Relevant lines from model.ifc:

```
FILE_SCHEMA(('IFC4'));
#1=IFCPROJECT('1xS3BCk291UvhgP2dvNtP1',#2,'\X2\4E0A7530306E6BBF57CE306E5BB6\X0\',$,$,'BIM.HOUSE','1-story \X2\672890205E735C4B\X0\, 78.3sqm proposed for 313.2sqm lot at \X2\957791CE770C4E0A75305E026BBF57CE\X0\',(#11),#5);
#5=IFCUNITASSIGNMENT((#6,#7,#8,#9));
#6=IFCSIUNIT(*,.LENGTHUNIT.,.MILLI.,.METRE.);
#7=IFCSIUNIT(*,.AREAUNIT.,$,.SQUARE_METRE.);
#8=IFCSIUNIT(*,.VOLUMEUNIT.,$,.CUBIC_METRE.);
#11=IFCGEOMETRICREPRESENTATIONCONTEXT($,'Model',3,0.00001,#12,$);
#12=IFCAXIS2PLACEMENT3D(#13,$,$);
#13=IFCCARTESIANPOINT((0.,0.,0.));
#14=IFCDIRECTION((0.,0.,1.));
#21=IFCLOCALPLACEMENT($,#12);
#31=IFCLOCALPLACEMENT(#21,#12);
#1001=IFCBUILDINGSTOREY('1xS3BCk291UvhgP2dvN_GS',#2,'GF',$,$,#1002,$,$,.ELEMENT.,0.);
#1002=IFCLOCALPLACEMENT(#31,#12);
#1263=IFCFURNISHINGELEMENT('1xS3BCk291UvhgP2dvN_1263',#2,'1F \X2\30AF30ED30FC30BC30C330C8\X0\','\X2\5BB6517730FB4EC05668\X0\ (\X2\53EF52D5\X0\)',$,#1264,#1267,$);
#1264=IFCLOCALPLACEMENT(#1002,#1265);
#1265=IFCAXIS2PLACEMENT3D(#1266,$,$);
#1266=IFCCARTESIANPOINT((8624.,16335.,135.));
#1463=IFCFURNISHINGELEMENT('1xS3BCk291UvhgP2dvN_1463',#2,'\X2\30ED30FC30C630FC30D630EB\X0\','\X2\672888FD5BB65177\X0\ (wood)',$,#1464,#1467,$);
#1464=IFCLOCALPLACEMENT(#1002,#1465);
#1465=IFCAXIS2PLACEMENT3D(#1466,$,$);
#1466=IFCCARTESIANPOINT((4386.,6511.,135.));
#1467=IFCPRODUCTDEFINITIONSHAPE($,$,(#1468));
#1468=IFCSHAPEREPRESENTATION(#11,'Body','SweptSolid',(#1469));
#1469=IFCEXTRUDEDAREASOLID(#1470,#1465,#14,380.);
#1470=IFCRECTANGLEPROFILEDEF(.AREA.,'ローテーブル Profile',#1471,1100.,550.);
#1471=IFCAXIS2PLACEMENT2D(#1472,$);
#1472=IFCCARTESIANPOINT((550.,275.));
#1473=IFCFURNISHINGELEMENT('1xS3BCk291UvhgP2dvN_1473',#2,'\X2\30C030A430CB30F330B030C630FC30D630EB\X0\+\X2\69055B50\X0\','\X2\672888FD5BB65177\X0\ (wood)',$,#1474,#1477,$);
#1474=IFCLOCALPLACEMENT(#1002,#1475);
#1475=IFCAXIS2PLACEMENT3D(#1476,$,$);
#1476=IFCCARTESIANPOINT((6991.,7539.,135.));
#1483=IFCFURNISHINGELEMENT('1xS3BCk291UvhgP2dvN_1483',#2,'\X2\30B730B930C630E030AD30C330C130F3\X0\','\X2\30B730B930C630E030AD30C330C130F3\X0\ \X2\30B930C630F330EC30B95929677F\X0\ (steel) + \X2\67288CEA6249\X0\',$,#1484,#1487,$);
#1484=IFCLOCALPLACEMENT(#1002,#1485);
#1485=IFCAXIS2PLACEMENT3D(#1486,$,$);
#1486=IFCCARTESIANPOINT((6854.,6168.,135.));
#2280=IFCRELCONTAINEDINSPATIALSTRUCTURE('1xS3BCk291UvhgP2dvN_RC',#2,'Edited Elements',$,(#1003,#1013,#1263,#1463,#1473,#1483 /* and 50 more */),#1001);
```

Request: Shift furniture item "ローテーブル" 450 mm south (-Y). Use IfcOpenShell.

```python
import ifcopenshell
import ifcopenshell.api.geometry
import ifcopenshell.util.placement
import ifcopenshell.util.unit

model = ifcopenshell.open("model.ifc")
unit_scale = ifcopenshell.util.unit.calculate_unit_scale(model)

item = model.by_id(1463)
matrix = ifcopenshell.util.placement.get_local_placement(item.ObjectPlacement)
matrix[1, 3] -= 0.45 / unit_scale
ifcopenshell.api.geometry.edit_object_placement(model, product=item, matrix=matrix, is_si=False)

print(ifcopenshell.util.placement.get_local_placement(item.ObjectPlacement).round(3) + 0.0)

model.write("model-out.ifc")
```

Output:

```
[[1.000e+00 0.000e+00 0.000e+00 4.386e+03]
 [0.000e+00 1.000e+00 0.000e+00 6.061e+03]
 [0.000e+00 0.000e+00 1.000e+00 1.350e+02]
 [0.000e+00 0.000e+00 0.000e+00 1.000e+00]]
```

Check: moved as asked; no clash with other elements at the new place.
